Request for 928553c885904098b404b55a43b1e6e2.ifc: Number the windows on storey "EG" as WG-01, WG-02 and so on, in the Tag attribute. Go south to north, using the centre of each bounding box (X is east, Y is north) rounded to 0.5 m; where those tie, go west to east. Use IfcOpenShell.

First a look at what the model holds.

```python
import ifcopenshell
import ifcopenshell.util.element
import ifcopenshell.util.placement

model = ifcopenshell.open("928553c885904098b404b55a43b1e6e2.ifc")
print(model.schema)
storey = next(s for s in model.by_type("IfcBuildingStorey") if s.Name == "EG")
windows = [e for e in ifcopenshell.util.element.get_decomposition(storey) if e.is_a("IfcWindow")]
for e in sorted(windows, key=lambda e: e.id()):
    origin = ifcopenshell.util.placement.get_local_placement(e.ObjectPlacement)[:3, 3]
    print(e.id(), e.Tag, e.Name, origin.round(2) + 0.0, sep=" | ")
```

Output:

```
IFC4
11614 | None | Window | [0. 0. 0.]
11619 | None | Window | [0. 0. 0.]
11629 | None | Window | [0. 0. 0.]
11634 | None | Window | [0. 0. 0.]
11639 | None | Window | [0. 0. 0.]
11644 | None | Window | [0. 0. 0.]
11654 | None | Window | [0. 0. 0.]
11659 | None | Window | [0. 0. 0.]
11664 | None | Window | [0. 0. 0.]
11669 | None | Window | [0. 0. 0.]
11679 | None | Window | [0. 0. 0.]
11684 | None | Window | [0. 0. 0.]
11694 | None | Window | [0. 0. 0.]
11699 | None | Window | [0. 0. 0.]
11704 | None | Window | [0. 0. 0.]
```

```python
import ifcopenshell
import ifcopenshell.geom
import ifcopenshell.util.element
import ifcopenshell.util.shape

model = ifcopenshell.open("928553c885904098b404b55a43b1e6e2.ifc")
settings = ifcopenshell.geom.settings()
settings.set("use-world-coords", True)


def centre(element):
    shape = ifcopenshell.geom.create_shape(settings, element)
    return ifcopenshell.util.shape.get_bbox_centroid(shape.geometry)


storey = next(s for s in model.by_type("IfcBuildingStorey") if s.Name == "EG")
windows = [e for e in ifcopenshell.util.element.get_decomposition(storey) if e.is_a("IfcWindow")]

# Insertion points can sit at a corner or the storey origin, so sort by the geometry (in metres).
centres = {e: centre(e) for e in windows}
windows.sort(key=lambda e: (round(centres[e][1] / 0.5), centres[e][0]))

for i, e in enumerate(windows, start=1):
    number = f"WG-{i:02d}"
    e.Tag = number
    print(e.id(), number)

model.write("928553c885904098b404b55a43b1e6e2_edited.ifc")
```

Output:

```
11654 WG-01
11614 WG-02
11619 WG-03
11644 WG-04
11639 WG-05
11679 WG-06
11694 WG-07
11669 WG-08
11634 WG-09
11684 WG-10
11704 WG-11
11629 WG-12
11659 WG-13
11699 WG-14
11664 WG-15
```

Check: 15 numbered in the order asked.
